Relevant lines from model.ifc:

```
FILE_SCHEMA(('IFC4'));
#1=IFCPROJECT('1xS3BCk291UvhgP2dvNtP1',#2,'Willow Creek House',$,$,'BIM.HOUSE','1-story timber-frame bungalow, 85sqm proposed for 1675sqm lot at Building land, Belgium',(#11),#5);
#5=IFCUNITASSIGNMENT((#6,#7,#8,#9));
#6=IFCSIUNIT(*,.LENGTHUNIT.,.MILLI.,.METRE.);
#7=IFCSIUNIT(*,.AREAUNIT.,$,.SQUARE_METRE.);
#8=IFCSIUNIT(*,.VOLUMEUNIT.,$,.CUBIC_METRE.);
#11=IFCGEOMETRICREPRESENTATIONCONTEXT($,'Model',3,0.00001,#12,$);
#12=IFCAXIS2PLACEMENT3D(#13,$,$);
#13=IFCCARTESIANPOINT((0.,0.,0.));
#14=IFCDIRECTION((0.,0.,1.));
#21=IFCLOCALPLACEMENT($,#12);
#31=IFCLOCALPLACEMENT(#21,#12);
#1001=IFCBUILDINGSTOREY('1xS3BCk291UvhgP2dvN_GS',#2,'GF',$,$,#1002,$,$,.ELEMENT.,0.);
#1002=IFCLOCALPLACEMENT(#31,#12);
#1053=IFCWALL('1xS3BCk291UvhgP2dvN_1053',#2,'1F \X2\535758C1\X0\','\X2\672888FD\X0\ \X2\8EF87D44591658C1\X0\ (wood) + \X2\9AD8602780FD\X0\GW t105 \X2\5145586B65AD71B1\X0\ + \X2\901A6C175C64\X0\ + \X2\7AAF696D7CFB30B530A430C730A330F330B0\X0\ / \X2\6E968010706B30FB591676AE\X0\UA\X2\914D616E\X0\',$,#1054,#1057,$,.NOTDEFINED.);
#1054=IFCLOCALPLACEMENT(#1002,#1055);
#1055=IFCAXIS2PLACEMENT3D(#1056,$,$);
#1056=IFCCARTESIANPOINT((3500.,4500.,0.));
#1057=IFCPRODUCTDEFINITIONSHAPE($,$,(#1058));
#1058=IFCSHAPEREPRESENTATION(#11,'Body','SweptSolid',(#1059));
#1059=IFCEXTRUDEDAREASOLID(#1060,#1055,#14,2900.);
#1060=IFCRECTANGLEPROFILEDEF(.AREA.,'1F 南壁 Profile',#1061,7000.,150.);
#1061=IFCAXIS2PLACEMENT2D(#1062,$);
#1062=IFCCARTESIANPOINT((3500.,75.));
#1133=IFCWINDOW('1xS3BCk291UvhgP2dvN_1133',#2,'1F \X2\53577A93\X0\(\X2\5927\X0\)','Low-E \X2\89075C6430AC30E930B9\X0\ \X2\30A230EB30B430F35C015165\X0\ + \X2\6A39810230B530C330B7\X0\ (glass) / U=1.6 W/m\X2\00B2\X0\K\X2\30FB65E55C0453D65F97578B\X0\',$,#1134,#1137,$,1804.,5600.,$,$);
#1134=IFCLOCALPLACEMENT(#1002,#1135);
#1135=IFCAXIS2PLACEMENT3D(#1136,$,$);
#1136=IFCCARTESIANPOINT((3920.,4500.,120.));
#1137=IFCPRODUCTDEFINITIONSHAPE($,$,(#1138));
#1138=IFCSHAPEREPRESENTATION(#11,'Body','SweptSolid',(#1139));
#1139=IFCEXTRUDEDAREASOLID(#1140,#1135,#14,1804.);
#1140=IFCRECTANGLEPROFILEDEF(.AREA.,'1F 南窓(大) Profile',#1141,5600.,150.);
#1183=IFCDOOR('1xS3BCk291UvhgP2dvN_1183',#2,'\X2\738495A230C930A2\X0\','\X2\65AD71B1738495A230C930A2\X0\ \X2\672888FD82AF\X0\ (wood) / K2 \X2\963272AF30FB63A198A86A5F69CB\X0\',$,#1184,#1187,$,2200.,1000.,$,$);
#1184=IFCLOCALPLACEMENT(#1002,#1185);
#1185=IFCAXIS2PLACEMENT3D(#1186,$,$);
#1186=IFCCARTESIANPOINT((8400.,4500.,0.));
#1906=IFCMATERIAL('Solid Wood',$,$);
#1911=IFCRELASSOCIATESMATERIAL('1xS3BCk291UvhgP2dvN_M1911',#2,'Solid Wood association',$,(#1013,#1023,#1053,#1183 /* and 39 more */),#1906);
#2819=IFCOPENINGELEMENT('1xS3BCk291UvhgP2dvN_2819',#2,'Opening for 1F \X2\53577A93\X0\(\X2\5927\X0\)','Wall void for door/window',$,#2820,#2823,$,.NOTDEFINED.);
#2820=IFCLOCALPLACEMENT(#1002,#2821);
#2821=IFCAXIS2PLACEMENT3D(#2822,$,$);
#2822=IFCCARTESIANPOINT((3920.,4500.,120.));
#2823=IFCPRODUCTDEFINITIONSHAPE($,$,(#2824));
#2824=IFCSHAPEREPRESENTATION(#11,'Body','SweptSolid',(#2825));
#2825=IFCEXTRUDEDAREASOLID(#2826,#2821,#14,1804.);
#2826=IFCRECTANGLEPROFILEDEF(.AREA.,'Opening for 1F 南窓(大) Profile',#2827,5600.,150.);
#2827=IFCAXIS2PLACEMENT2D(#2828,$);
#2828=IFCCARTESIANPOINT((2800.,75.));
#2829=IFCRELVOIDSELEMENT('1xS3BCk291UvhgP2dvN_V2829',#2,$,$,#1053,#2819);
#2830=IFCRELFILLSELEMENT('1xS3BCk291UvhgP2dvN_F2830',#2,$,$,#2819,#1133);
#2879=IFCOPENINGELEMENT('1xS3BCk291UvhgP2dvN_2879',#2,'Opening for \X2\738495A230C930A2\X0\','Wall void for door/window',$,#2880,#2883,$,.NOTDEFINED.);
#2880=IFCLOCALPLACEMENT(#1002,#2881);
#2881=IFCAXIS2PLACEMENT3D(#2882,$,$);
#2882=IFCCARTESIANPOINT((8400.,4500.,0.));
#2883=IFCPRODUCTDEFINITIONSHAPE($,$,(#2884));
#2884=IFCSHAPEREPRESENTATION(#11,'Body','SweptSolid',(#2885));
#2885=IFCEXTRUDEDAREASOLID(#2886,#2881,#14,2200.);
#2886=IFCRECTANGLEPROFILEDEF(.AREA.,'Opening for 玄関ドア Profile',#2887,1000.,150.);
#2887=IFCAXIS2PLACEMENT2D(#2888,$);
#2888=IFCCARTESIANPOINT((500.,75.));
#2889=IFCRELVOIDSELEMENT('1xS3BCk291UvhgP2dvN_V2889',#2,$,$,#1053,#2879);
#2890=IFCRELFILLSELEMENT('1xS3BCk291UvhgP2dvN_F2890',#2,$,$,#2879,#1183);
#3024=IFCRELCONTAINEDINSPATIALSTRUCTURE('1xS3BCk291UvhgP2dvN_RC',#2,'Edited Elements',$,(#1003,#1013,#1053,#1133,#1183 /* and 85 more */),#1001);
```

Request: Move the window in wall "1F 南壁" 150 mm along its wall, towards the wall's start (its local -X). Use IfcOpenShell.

```python
import ifcopenshell
import ifcopenshell.api.geometry
import ifcopenshell.util.placement

model = ifcopenshell.open("model.ifc")

window = model.by_guid("1xS3BCk291UvhgP2dvN_1133")
opening = window.FillsVoids[0].RelatingOpeningElement
wall = opening.VoidsElements[0].RelatingBuildingElement

wall_matrix = ifcopenshell.util.placement.get_local_placement(wall.ObjectPlacement)
shift = wall_matrix[:3, 0] * -150.0
before = ifcopenshell.util.placement.get_local_placement(window.ObjectPlacement)[:3, 3].copy()

# The window is not placed relative to its opening, so move both.
for product in (opening, window):
    matrix = ifcopenshell.util.placement.get_local_placement(product.ObjectPlacement)
    matrix[:3, 3] += shift
    ifcopenshell.api.geometry.edit_object_placement(model, product=product, matrix=matrix, is_si=False)

after = ifcopenshell.util.placement.get_local_placement(window.ObjectPlacement)[:3, 3]
print("window moved by", (after - before).round(3) + 0.0)

model.write("model_v2.ifc")
```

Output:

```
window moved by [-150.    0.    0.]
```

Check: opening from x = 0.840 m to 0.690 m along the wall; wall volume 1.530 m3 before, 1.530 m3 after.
